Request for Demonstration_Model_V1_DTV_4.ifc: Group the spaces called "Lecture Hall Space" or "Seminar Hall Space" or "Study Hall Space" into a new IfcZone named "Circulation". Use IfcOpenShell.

First a look at what the model holds.

```python
import ifcopenshell

model = ifcopenshell.open("Demonstration_Model_V1_DTV_4.ifc")
print(model.schema)
seen = {}
for space in model.by_type("IfcSpace"):
    seen[space.LongName] = seen.get(space.LongName, 0) + 1
for name, count in sorted(seen.items(), key=str):
    print(count, "x", name)
print("zones:", [z.Name for z in model.by_type("IfcZone")][:20])
```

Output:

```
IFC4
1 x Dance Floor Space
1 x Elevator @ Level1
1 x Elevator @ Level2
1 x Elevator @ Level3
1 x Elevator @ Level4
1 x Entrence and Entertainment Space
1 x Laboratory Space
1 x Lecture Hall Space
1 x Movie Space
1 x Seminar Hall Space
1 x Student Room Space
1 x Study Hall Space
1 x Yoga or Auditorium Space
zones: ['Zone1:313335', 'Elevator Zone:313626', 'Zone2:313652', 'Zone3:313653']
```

```python
import ifcopenshell
import ifcopenshell.api.group
import ifcopenshell.api.root

model = ifcopenshell.open("Demonstration_Model_V1_DTV_4.ifc")

names = {"Lecture Hall Space", "Seminar Hall Space", "Study Hall Space"}
spaces = [s for s in model.by_type("IfcSpace") if s.LongName in names]

zone = ifcopenshell.api.root.create_entity(model, ifc_class="IfcZone", name="Circulation")
ifcopenshell.api.group.assign_group(model, products=spaces, group=zone)
print(len(spaces), "spaces in", zone.Name)

model.write("Demonstration_Model_V1_DTV_4_v2.ifc")
```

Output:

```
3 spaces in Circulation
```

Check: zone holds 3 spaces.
